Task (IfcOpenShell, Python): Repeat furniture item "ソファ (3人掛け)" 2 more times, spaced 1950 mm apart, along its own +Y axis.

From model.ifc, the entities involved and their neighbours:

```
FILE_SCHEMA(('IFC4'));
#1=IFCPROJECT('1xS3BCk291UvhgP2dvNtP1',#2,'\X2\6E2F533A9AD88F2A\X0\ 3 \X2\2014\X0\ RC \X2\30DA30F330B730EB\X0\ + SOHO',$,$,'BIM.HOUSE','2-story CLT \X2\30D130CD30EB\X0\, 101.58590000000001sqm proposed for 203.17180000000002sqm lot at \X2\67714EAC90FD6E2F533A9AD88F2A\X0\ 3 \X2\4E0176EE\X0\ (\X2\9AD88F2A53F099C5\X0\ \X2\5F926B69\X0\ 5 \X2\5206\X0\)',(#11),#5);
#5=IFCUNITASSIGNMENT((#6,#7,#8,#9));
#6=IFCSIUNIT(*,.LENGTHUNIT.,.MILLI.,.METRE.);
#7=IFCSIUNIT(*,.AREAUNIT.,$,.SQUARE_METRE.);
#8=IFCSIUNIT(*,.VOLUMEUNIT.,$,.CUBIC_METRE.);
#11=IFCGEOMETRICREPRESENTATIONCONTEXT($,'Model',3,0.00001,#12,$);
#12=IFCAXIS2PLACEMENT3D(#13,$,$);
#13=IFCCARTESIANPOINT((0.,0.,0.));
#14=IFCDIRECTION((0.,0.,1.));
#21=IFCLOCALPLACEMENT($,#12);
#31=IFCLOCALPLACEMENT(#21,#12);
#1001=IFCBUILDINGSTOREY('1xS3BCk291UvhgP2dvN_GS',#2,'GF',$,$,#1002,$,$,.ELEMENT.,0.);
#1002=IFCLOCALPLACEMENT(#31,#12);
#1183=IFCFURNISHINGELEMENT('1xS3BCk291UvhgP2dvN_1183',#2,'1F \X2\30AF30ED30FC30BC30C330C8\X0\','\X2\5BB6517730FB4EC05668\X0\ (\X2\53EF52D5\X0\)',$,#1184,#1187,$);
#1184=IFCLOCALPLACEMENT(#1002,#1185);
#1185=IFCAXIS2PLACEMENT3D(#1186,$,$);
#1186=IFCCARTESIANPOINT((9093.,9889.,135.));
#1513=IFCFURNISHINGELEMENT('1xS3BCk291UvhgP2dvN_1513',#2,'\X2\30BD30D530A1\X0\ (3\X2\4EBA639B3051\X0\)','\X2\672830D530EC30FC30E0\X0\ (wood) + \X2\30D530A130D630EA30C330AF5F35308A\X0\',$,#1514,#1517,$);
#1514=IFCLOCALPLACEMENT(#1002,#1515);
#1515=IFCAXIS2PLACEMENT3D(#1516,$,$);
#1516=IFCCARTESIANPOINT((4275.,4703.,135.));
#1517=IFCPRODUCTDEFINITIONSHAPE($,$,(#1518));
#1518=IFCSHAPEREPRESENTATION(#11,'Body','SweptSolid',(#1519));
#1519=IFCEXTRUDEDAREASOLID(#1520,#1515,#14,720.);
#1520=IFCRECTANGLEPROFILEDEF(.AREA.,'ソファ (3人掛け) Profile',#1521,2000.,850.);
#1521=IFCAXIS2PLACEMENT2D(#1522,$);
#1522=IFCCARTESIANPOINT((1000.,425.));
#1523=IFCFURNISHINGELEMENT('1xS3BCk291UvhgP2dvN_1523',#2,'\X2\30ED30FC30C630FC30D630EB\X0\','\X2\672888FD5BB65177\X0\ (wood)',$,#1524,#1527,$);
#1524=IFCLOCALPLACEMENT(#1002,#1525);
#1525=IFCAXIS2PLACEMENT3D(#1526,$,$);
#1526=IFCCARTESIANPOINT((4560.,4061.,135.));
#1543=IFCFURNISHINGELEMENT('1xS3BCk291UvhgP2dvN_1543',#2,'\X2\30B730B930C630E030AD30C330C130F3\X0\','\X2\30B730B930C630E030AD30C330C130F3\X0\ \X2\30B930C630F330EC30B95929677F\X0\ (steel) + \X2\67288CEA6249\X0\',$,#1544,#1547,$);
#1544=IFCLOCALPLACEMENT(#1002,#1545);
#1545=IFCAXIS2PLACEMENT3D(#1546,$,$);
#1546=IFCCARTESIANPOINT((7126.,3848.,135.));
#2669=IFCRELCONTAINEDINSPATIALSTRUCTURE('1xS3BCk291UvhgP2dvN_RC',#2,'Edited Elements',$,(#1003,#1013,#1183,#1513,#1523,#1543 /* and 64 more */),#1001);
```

```python
import ifcopenshell
import ifcopenshell.api.geometry
import ifcopenshell.api.root
import ifcopenshell.util.element
import ifcopenshell.util.placement

model = ifcopenshell.open("model.ifc")


def reuse_history(source, copy):
    """copy_class also copies each property set's owner history, people and application; keep the originals."""
    for rel in copy.IsDefinedBy:
        if rel.is_a("IfcRelDefinesByProperties") and (history := rel.RelatingPropertyDefinition.OwnerHistory):
            rel.RelatingPropertyDefinition.OwnerHistory = source.OwnerHistory
            ifcopenshell.util.element.remove_deep2(model, history)


source = model.by_guid("1xS3BCk291UvhgP2dvN_1513")
base = ifcopenshell.util.placement.get_local_placement(source.ObjectPlacement)
step = base[:3, 1] * 1950.0

for i in range(1, 3):
    copy = ifcopenshell.api.root.copy_class(model, product=source)
    copy.Representation = ifcopenshell.util.element.copy_deep(
        model, source.Representation, exclude=["IfcGeometricRepresentationContext", "IfcRepresentationMap"]
    )
    reuse_history(source, copy)
    matrix = base.copy()
    matrix[:3, 3] += i * step
    print("added at", matrix[:3, 3].round(3) + 0.0)
    ifcopenshell.api.geometry.edit_object_placement(model, product=copy, matrix=matrix, is_si=False)

model.write("model-out.ifc")
```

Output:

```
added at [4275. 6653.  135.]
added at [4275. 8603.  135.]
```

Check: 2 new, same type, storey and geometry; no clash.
